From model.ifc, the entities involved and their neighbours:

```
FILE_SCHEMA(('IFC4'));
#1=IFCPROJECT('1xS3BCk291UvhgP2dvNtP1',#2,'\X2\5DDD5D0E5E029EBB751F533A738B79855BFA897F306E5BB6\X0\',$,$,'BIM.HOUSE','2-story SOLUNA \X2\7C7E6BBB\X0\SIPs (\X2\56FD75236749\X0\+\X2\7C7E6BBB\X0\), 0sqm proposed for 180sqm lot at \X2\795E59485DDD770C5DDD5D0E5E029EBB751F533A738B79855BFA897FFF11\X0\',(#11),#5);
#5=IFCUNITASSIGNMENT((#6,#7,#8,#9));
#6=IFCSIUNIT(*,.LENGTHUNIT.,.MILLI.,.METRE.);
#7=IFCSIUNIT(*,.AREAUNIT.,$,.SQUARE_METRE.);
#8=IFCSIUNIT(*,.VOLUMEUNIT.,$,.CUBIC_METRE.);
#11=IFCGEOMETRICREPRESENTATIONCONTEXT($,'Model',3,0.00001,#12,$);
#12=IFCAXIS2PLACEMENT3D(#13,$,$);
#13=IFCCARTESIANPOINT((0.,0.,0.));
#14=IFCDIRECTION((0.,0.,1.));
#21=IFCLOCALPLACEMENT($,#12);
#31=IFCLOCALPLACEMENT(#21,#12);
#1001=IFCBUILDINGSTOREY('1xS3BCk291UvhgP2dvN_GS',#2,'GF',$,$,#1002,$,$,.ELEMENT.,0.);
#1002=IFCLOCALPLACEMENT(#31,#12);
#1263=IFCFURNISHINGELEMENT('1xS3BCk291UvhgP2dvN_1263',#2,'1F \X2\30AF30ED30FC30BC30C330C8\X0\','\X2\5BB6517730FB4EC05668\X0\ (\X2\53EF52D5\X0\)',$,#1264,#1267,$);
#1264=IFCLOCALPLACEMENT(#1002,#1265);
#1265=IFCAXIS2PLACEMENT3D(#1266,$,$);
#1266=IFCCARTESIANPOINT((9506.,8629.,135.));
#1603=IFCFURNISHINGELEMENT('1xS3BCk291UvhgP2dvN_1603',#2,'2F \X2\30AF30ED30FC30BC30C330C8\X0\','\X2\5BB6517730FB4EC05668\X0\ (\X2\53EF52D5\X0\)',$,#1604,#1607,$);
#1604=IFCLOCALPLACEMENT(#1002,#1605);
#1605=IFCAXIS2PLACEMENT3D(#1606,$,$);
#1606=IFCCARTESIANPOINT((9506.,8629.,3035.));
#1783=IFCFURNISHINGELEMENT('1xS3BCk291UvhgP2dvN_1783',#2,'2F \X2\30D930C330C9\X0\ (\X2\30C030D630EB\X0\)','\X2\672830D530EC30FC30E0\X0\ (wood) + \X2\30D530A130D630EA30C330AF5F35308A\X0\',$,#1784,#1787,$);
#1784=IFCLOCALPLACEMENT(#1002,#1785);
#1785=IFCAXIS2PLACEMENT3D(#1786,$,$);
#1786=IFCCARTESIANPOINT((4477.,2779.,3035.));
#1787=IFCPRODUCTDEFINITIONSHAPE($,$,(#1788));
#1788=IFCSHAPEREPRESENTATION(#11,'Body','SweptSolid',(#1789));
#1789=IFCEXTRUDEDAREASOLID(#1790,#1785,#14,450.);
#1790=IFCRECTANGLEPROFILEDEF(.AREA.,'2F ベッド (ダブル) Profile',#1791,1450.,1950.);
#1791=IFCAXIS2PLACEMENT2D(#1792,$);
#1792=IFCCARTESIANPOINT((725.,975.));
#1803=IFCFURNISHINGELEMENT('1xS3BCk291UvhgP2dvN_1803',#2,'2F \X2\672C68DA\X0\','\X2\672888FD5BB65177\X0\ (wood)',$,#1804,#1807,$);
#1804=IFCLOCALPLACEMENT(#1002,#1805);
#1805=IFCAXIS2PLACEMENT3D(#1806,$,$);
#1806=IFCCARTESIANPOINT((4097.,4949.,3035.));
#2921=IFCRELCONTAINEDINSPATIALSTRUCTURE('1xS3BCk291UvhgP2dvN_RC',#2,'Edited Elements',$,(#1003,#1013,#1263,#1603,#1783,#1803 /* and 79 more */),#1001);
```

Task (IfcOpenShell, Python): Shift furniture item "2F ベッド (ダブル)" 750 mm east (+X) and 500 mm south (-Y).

```python
import ifcopenshell
import ifcopenshell.api.geometry
import ifcopenshell.util.placement
import ifcopenshell.util.unit

model = ifcopenshell.open("model.ifc")
unit_scale = ifcopenshell.util.unit.calculate_unit_scale(model)

item = model.by_id(1783)
matrix = ifcopenshell.util.placement.get_local_placement(item.ObjectPlacement)
matrix[0, 3] += 0.75 / unit_scale
matrix[1, 3] -= 0.5 / unit_scale
ifcopenshell.api.geometry.edit_object_placement(model, product=item, matrix=matrix, is_si=False)

print(ifcopenshell.util.placement.get_local_placement(item.ObjectPlacement).round(3) + 0.0)

model.write("model-out.ifc")
```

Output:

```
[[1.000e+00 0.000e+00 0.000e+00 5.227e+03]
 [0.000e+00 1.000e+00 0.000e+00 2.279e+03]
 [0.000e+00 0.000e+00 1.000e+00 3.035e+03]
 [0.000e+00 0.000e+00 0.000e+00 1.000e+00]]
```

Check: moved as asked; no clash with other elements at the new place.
